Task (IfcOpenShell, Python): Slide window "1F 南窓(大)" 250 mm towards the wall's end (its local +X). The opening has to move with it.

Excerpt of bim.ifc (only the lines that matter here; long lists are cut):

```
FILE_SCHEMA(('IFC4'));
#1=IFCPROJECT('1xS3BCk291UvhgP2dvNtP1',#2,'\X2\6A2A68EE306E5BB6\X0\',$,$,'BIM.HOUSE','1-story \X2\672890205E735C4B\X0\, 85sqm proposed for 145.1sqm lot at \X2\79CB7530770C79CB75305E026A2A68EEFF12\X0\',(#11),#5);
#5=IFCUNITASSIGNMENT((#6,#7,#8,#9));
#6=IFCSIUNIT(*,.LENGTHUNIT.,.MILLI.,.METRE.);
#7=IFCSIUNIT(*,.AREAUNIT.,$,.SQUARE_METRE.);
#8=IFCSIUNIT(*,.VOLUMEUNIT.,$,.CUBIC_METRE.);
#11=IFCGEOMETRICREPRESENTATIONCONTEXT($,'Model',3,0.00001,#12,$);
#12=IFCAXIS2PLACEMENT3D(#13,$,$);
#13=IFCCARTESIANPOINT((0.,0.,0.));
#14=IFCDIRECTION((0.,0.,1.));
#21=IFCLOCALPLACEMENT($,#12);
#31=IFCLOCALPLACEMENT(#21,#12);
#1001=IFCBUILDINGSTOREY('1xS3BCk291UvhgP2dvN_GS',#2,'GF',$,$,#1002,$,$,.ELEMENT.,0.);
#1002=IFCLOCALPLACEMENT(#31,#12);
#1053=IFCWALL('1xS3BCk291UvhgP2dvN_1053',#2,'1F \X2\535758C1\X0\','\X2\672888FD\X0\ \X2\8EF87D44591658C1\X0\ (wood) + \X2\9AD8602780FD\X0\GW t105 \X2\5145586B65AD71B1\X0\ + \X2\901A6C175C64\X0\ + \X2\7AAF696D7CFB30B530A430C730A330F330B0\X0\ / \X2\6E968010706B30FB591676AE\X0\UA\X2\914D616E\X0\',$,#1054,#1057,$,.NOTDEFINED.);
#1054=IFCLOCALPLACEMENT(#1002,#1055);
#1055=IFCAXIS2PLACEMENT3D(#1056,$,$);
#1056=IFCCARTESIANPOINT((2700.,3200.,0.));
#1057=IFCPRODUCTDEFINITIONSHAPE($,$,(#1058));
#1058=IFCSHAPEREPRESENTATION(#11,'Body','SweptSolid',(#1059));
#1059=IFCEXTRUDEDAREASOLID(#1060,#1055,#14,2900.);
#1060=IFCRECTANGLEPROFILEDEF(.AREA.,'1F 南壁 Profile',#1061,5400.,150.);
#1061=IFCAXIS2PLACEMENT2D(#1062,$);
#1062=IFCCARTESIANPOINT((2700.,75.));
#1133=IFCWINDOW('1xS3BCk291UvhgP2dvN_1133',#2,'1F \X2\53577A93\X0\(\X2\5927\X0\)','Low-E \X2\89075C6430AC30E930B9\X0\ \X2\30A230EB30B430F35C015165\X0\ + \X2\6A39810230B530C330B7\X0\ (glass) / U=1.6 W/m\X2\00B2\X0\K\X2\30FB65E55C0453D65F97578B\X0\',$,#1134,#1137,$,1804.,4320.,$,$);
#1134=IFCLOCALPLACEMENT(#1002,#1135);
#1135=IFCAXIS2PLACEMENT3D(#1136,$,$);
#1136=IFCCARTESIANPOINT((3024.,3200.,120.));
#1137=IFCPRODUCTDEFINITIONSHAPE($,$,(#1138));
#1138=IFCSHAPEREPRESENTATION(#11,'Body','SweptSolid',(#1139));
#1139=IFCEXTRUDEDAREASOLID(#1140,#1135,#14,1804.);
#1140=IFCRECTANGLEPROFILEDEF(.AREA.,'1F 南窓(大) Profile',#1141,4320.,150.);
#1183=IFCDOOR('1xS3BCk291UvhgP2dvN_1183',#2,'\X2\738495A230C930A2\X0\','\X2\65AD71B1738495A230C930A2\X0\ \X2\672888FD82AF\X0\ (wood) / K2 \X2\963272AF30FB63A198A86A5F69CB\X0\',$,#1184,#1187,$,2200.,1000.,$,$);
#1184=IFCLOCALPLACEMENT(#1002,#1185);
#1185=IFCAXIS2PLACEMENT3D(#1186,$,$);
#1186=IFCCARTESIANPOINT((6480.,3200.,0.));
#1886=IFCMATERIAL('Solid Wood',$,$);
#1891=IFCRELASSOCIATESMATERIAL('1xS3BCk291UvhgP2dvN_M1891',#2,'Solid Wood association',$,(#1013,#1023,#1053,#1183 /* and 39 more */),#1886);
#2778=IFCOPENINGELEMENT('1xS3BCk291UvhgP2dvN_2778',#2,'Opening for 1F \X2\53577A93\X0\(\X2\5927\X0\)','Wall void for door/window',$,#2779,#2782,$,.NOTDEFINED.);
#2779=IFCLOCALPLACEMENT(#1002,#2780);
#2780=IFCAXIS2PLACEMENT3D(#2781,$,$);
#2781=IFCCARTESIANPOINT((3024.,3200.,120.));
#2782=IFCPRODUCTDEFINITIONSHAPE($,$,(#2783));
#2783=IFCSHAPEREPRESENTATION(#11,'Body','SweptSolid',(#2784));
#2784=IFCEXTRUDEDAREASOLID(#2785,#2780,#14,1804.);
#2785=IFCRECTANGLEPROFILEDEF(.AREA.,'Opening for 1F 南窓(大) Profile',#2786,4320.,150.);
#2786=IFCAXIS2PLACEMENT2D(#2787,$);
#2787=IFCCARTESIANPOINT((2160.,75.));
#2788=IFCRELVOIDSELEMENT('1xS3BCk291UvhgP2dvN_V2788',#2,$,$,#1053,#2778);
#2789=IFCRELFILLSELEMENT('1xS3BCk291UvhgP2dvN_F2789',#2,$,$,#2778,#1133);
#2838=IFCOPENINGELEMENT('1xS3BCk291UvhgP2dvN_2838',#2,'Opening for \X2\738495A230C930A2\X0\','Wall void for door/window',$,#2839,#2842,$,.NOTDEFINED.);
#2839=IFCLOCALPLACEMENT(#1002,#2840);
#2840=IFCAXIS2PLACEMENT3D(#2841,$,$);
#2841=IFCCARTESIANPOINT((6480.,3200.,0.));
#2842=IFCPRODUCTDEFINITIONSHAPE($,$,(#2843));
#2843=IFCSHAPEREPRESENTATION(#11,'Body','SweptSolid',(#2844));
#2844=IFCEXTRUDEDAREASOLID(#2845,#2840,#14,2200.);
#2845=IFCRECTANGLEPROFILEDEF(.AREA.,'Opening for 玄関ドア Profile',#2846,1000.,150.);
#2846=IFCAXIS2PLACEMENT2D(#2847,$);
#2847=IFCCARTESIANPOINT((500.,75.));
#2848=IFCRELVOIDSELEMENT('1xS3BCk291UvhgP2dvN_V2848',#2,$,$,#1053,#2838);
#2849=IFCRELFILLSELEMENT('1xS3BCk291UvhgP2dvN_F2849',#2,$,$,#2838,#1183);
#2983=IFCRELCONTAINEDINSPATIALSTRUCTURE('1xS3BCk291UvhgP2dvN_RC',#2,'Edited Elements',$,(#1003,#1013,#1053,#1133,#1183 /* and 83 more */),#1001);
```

```python
import ifcopenshell
import ifcopenshell.api.geometry
import ifcopenshell.util.placement

model = ifcopenshell.open("bim.ifc")

window = model.by_id(1133)
opening = window.FillsVoids[0].RelatingOpeningElement
wall = opening.VoidsElements[0].RelatingBuildingElement

wall_matrix = ifcopenshell.util.placement.get_local_placement(wall.ObjectPlacement)
shift = wall_matrix[:3, 0] * 250.0
before = ifcopenshell.util.placement.get_local_placement(window.ObjectPlacement)[:3, 3].copy()

# The window is not placed relative to its opening, so move both.
for product in (opening, window):
    matrix = ifcopenshell.util.placement.get_local_placement(product.ObjectPlacement)
    matrix[:3, 3] += shift
    ifcopenshell.api.geometry.edit_object_placement(model, product=product, matrix=matrix, is_si=False)

after = ifcopenshell.util.placement.get_local_placement(window.ObjectPlacement)[:3, 3]
print("window moved by", (after - before).round(3) + 0.0)

model.write("bim_edited.ifc")
```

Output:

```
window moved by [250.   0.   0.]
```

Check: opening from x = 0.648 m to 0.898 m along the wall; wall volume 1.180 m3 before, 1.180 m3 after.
